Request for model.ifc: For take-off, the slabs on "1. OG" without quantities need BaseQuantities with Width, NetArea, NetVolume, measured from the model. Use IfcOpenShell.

First a look at what the model holds.

```python
import ifcopenshell
import ifcopenshell.util.element
import ifcopenshell.util.unit

model = ifcopenshell.open("model.ifc")
print(model.schema)
for unit_type in ("LENGTHUNIT", "AREAUNIT", "VOLUMEUNIT"):
    print(unit_type, ifcopenshell.util.unit.calculate_unit_scale(model, unit_type))
storey = next(s for s in model.by_type("IfcBuildingStorey") if s.Name == "1. OG")
slabs = [e for e in ifcopenshell.util.element.get_decomposition(storey) if e.is_a("IfcSlab")]
for e in sorted(slabs, key=lambda e: e.id()):
    print(e.id(), e.is_a(), e.Name, list(ifcopenshell.util.element.get_psets(e, qtos_only=True)), sep=" | ")
```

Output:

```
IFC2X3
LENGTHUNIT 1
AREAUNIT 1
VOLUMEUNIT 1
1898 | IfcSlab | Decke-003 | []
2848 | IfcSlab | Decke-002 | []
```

```python
import ifcopenshell
import ifcopenshell.api.pset
import ifcopenshell.geom
import ifcopenshell.util.element
import ifcopenshell.util.shape
import ifcopenshell.util.unit

model = ifcopenshell.open("model.ifc")
unit_scale = ifcopenshell.util.unit.calculate_unit_scale(model)
area_scale = ifcopenshell.util.unit.calculate_unit_scale(model, "AREAUNIT")
volume_scale = ifcopenshell.util.unit.calculate_unit_scale(model, "VOLUMEUNIT")
settings = ifcopenshell.geom.settings()

storey = next(s for s in model.by_type("IfcBuildingStorey") if s.Name == "1. OG")
slabs = [e for e in ifcopenshell.util.element.get_decomposition(storey) if e.is_a("IfcSlab")]

for e in sorted(slabs, key=lambda e: e.id()):
    if ifcopenshell.util.element.get_psets(e, qtos_only=True, should_inherit=False):
        continue
    # Geometry comes back in metres, in the element's own axes.
    shape = ifcopenshell.geom.create_shape(settings, e)
    values = {
        "Width": ifcopenshell.util.shape.get_z(shape.geometry) / unit_scale,
        "NetArea": ifcopenshell.util.shape.get_footprint_area(shape.geometry) / area_scale,
        "NetVolume": ifcopenshell.util.shape.get_volume(shape.geometry) / volume_scale,
    }
    qto = ifcopenshell.api.pset.add_qto(model, product=e, name="BaseQuantities")
    ifcopenshell.api.pset.edit_qto(model, qto=qto, properties=values)
    print(e.id(), {k: round(v, 3) for k, v in values.items()})

model.write("model_edited.ifc")
```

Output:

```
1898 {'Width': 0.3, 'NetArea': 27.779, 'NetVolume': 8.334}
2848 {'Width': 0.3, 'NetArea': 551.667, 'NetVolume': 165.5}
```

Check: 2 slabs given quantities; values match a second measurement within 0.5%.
